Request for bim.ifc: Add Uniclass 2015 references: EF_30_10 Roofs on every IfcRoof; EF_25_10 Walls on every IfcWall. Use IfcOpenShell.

First a look at what the model holds.

```python
import ifcopenshell

model = ifcopenshell.open("bim.ifc")
print(model.schema)
print("classifications:", [c.Name for c in model.by_type("IfcClassification")])
for ifc_class in ("IfcDoor", "IfcRoof", "IfcStair", "IfcWall", "IfcWindow"):
    print(ifc_class, len(model.by_type(ifc_class)))
```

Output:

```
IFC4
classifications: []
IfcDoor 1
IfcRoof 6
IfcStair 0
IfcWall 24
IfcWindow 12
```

```python
import ifcopenshell
import ifcopenshell.api.classification

model = ifcopenshell.open("bim.ifc")

system = ifcopenshell.api.classification.add_classification(model, classification="Uniclass 2015")

codes = {
    "IfcRoof": ("EF_30_10", "Roofs"),
    "IfcWall": ("EF_25_10", "Walls"),
}
for ifc_class, (code, name) in codes.items():
    products = model.by_type(ifc_class)
    ifcopenshell.api.classification.add_reference(
        model, products=products, classification=system, identification=code, name=name
    )
    print(code, len(products))

model.write("bim-out.ifc")
```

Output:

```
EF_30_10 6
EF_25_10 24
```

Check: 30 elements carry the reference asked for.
